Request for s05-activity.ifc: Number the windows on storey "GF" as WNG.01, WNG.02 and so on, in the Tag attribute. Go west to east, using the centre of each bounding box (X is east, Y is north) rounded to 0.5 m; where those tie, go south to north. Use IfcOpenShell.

First a look at what the model holds.

```python
import ifcopenshell
import ifcopenshell.util.element
import ifcopenshell.util.placement

model = ifcopenshell.open("s05-activity.ifc")
print(model.schema)
storey = next(s for s in model.by_type("IfcBuildingStorey") if s.Name == "GF")
windows = [e for e in ifcopenshell.util.element.get_decomposition(storey) if e.is_a("IfcWindow")]
for e in sorted(windows, key=lambda e: e.id()):
    origin = ifcopenshell.util.placement.get_local_placement(e.ObjectPlacement)[:3, 3]
    print(e.id(), e.Tag, e.Name, origin.round(2) + 0.0, sep=" | ")
```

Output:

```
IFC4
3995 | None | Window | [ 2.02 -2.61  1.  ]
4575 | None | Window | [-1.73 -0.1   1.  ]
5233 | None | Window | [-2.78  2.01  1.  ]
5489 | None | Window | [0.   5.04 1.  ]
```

```python
import ifcopenshell
import ifcopenshell.geom
import ifcopenshell.util.element
import ifcopenshell.util.shape

model = ifcopenshell.open("s05-activity.ifc")
settings = ifcopenshell.geom.settings()
settings.set("use-world-coords", True)


def centre(element):
    shape = ifcopenshell.geom.create_shape(settings, element)
    return ifcopenshell.util.shape.get_bbox_centroid(shape.geometry)


storey = next(s for s in model.by_type("IfcBuildingStorey") if s.Name == "GF")
windows = [e for e in ifcopenshell.util.element.get_decomposition(storey) if e.is_a("IfcWindow")]

# Insertion points can sit at a corner or the storey origin, so sort by the geometry (in metres).
centres = {e: centre(e) for e in windows}
windows.sort(key=lambda e: (round(centres[e][0] / 0.5), centres[e][1]))

for i, e in enumerate(windows, start=1):
    number = f"WNG.{i:02d}"
    e.Tag = number
    print(e.id(), number)

model.write("s05-activity_updated.ifc")
```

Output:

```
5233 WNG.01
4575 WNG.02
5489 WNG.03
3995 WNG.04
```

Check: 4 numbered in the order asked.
